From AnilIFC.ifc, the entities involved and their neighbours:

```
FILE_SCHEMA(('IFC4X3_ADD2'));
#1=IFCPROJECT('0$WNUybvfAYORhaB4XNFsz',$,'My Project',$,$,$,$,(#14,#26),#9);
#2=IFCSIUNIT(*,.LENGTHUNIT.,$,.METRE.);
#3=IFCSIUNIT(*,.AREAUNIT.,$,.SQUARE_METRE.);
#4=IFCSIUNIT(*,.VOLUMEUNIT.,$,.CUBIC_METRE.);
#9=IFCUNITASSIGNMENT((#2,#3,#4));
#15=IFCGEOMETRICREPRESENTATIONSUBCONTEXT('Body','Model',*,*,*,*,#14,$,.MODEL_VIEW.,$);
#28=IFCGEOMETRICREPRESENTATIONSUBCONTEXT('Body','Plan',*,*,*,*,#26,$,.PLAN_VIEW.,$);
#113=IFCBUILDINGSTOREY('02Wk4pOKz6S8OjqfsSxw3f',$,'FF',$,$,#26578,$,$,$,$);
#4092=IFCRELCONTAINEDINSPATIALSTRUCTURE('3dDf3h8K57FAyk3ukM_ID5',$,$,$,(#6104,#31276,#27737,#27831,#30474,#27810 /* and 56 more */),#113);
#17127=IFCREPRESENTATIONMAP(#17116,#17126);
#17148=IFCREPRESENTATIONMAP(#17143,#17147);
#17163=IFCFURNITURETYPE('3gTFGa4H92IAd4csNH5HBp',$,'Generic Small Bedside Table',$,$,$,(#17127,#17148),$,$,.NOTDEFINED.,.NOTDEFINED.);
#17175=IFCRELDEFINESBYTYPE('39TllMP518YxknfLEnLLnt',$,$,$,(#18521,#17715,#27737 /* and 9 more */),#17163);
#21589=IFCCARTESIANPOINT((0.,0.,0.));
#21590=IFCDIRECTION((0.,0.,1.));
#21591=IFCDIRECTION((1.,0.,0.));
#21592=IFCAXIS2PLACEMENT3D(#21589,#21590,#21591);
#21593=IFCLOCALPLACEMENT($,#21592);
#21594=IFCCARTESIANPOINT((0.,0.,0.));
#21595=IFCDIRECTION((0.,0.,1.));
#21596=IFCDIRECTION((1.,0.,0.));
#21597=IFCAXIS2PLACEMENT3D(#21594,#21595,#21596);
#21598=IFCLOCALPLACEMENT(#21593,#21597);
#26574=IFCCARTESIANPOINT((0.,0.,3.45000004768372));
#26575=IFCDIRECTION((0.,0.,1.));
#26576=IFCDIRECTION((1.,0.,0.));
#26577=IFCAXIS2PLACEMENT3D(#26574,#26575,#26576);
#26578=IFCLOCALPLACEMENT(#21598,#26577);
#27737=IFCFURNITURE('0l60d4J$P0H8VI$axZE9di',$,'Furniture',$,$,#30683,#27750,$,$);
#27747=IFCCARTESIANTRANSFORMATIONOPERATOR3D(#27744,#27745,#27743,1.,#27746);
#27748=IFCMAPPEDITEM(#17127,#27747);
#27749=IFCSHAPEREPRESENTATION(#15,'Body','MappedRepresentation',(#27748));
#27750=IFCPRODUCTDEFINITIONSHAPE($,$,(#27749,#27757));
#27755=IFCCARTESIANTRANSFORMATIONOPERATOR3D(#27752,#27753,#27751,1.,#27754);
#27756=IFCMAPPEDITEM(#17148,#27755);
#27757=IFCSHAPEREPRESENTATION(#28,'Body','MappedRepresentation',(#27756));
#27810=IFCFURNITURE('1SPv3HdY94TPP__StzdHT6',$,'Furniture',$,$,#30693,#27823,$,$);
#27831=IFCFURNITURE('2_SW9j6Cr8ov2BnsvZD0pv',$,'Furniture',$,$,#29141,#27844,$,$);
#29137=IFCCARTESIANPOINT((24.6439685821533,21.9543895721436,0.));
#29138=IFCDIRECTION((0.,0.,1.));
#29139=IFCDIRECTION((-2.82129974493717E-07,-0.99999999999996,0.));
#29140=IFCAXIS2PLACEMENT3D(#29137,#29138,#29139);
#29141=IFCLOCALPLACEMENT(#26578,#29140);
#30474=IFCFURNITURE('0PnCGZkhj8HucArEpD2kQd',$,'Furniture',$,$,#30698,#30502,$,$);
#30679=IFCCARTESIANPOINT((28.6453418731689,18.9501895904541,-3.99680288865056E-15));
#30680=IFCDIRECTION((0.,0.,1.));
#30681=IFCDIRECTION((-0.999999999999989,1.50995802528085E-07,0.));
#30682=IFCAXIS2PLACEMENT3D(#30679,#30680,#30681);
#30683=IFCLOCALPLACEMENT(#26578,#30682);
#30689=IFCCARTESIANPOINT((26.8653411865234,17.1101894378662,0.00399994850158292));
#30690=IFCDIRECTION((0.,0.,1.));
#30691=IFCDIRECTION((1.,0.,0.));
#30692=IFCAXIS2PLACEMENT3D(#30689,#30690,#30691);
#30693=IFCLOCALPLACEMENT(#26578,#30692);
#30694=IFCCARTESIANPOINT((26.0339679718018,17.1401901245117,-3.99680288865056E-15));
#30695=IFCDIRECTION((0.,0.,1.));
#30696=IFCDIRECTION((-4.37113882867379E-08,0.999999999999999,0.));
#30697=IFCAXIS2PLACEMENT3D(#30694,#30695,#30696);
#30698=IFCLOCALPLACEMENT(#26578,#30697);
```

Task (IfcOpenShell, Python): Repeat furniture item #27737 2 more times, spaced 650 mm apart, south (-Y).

```python
import numpy as np
import ifcopenshell
import ifcopenshell.api.geometry
import ifcopenshell.api.root
import ifcopenshell.util.element
import ifcopenshell.util.placement
import ifcopenshell.util.unit

model = ifcopenshell.open("AnilIFC.ifc")
unit_scale = ifcopenshell.util.unit.calculate_unit_scale(model)

source = model.by_guid("0l60d4J$P0H8VI$axZE9di")
base = ifcopenshell.util.placement.get_local_placement(source.ObjectPlacement)
step = np.array([0.0, -1.0, 0.0]) * 0.65 / unit_scale

for i in range(1, 3):
    copy = ifcopenshell.api.root.copy_class(model, product=source)
    copy.Representation = ifcopenshell.util.element.copy_deep(
        model, source.Representation, exclude=["IfcGeometricRepresentationContext", "IfcRepresentationMap"]
    )
    matrix = base.copy()
    matrix[:3, 3] += i * step
    print("added at", matrix[:3, 3].round(3) + 0.0)
    ifcopenshell.api.geometry.edit_object_placement(model, product=copy, matrix=matrix, is_si=False)

model.write("AnilIFC_v2.ifc")
```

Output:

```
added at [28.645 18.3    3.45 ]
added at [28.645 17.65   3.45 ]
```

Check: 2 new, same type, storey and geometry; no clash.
